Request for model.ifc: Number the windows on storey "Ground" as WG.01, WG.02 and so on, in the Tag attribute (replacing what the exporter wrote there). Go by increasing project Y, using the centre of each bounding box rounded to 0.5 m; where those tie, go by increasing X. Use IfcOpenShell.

First a look at what the model holds.

```python
import ifcopenshell
import ifcopenshell.util.element
import ifcopenshell.util.placement

model = ifcopenshell.open("model.ifc")
print(model.schema)
storey = next(s for s in model.by_type("IfcBuildingStorey") if s.Name == "Ground")
windows = [e for e in ifcopenshell.util.element.get_decomposition(storey) if e.is_a("IfcWindow")]
for e in sorted(windows, key=lambda e: e.id()):
    origin = ifcopenshell.util.placement.get_local_placement(e.ObjectPlacement)[:3, 3]
    print(e.id(), e.Tag, e.Name, origin.round(2) + 0.0, sep=" | ")
```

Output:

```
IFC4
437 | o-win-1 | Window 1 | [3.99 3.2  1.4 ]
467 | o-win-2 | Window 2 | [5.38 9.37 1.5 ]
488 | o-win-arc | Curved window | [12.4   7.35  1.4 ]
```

```python
import ifcopenshell
import ifcopenshell.geom
import ifcopenshell.util.element
import ifcopenshell.util.shape

model = ifcopenshell.open("model.ifc")
settings = ifcopenshell.geom.settings()
settings.set("use-world-coords", True)


def centre(element):
    shape = ifcopenshell.geom.create_shape(settings, element)
    return ifcopenshell.util.shape.get_bbox_centroid(shape.geometry)


storey = next(s for s in model.by_type("IfcBuildingStorey") if s.Name == "Ground")
windows = [e for e in ifcopenshell.util.element.get_decomposition(storey) if e.is_a("IfcWindow")]

# Insertion points can sit at a corner or the storey origin, so sort by the geometry (in metres).
centres = {e: centre(e) for e in windows}
windows.sort(key=lambda e: (round(centres[e][1] / 0.5), centres[e][0]))

for i, e in enumerate(windows, start=1):
    number = f"WG.{i:02d}"
    e.Tag = number
    print(e.id(), number)

model.write("model_rev.ifc")
```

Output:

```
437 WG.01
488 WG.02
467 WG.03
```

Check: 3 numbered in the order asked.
